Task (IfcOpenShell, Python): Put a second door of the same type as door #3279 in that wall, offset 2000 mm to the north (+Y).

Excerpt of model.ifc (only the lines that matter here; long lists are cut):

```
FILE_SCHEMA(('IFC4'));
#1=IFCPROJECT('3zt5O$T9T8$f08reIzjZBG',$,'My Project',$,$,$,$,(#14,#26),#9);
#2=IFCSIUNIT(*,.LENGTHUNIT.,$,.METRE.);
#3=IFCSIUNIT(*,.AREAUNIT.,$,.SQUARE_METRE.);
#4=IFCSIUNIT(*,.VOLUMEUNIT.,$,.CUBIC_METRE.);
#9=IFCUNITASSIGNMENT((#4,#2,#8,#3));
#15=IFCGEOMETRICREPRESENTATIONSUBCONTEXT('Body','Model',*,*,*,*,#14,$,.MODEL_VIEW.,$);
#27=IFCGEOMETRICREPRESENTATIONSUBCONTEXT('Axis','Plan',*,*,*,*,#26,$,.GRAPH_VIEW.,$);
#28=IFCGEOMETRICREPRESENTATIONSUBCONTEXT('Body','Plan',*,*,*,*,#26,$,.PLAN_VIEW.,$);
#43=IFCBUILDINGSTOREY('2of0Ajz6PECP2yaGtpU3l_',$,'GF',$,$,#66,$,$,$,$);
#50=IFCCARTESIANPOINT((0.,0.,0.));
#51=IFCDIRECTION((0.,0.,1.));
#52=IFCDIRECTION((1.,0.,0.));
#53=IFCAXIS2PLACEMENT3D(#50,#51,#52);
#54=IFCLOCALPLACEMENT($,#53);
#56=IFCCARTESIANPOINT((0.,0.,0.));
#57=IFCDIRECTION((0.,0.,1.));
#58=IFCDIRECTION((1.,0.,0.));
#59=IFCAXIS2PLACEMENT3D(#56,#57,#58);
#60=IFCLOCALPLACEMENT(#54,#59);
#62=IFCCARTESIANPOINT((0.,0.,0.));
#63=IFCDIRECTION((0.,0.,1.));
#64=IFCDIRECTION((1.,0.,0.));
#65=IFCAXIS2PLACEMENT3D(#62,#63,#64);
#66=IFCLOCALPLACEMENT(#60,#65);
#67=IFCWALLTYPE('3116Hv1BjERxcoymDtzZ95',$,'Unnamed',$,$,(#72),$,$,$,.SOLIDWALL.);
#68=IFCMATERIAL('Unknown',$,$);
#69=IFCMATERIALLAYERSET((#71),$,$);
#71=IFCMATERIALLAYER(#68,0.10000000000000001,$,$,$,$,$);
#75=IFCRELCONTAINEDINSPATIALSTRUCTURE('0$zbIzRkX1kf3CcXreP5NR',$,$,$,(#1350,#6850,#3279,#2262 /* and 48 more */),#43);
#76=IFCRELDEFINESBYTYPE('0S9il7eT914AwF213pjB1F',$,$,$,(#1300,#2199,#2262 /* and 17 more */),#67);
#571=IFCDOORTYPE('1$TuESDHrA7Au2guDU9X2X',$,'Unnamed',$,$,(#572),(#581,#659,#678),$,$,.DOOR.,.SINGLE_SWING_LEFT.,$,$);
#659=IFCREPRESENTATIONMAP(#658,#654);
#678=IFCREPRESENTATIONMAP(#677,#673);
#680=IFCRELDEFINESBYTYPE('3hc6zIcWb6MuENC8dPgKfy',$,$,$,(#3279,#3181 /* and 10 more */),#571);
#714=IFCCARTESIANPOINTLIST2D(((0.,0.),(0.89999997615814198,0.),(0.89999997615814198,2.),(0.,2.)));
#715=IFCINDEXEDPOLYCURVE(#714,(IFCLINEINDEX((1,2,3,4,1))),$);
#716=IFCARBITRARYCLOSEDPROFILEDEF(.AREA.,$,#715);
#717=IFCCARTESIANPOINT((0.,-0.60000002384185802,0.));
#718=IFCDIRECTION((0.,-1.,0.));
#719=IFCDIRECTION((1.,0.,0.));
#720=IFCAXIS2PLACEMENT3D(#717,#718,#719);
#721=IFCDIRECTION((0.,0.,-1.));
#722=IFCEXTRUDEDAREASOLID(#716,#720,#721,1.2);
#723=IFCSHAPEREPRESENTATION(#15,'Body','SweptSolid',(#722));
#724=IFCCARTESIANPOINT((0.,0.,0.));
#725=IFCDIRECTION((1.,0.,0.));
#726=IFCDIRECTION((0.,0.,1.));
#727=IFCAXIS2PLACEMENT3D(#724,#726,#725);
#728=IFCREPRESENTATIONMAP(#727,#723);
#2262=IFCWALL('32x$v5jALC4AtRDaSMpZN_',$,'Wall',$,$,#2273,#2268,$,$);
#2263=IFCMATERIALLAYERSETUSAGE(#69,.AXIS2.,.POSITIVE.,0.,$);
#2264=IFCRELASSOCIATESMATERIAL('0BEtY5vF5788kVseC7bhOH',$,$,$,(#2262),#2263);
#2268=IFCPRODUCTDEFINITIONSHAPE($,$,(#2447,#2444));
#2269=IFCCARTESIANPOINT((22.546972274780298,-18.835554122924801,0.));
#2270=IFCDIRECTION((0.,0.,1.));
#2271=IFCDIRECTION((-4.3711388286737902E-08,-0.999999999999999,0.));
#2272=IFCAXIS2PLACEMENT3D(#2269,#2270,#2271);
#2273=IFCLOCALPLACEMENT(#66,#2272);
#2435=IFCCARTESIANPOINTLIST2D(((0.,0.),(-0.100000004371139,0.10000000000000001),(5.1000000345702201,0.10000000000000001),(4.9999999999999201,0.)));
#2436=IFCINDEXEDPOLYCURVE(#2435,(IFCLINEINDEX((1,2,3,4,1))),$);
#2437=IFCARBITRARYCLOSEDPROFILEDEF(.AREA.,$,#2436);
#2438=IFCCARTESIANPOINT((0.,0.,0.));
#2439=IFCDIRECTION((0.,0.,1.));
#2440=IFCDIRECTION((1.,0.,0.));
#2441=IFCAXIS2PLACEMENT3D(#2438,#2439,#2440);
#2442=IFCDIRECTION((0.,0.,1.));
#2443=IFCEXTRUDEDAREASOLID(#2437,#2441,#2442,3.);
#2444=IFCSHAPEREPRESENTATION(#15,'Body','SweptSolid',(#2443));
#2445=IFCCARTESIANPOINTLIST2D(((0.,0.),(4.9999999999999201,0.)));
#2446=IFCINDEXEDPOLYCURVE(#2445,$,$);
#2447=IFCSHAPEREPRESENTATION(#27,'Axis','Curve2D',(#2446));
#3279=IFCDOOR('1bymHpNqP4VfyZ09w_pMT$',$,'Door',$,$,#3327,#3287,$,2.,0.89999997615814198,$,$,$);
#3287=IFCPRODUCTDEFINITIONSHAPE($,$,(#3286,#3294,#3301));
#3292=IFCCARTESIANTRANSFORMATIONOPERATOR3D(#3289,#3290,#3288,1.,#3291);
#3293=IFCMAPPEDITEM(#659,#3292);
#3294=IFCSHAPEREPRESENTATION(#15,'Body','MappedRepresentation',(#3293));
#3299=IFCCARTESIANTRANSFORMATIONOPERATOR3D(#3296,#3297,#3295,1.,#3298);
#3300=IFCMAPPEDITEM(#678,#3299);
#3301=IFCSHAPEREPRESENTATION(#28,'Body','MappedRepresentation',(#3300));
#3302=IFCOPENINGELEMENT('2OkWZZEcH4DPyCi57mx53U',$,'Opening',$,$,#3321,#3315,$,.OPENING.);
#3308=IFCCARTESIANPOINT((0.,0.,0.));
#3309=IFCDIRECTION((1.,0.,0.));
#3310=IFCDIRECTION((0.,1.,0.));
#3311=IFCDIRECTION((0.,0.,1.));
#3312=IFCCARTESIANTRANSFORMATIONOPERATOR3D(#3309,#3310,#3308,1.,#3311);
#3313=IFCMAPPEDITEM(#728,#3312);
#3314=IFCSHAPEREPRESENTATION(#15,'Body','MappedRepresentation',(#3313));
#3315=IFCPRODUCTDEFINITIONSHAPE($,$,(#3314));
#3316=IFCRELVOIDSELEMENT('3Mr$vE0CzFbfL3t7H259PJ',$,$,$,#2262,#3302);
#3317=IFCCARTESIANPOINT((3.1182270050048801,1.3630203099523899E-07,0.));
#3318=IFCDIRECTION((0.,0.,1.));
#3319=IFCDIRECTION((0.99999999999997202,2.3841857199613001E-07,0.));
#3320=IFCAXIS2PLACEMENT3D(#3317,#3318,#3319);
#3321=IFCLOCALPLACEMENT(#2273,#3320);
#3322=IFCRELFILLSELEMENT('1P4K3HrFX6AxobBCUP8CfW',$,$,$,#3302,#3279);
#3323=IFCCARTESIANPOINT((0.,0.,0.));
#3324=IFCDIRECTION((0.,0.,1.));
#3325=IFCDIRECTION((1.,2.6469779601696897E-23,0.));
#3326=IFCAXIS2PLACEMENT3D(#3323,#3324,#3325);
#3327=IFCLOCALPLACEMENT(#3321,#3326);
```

```python
import ifcopenshell
import ifcopenshell.api.feature
import ifcopenshell.api.geometry
import ifcopenshell.api.root
import ifcopenshell.geom
import ifcopenshell.util.element
import ifcopenshell.util.placement
import ifcopenshell.util.shape

model = ifcopenshell.open("model.ifc")
settings = ifcopenshell.geom.settings()


def volume(element):
    """Net volume in cubic metres, openings subtracted."""
    shape = ifcopenshell.geom.create_shape(settings, element)
    return ifcopenshell.util.shape.get_volume(shape.geometry)


door = model.by_id(3279)
opening = door.FillsVoids[0].RelatingOpeningElement
wall = opening.VoidsElements[0].RelatingBuildingElement
before = volume(wall)
shift = ifcopenshell.util.placement.get_local_placement(wall.ObjectPlacement)[:3, 0] * -2.0

# copy_class copies the void relationship, type, container and properties, but no geometry.
new_opening = ifcopenshell.api.root.copy_class(model, product=opening)
new_opening.Representation = ifcopenshell.util.element.copy_deep(
    model, opening.Representation, exclude=["IfcGeometricRepresentationContext", "IfcRepresentationMap"]
)
new_door = ifcopenshell.api.root.copy_class(model, product=door)
new_door.Representation = ifcopenshell.util.element.copy_deep(
    model, door.Representation, exclude=["IfcGeometricRepresentationContext", "IfcRepresentationMap"]
)
ifcopenshell.api.feature.add_filling(model, opening=new_opening, element=new_door)

for old, new in ((opening, new_opening), (door, new_door)):
    matrix = ifcopenshell.util.placement.get_local_placement(old.ObjectPlacement)
    matrix[:3, 3] += shift
    ifcopenshell.api.geometry.edit_object_placement(model, product=new, matrix=matrix, is_si=False)

after = volume(wall)

print(f"wall volume {before:.3f} -> {after:.3f} m3")

model.write("model_edited.ifc")
```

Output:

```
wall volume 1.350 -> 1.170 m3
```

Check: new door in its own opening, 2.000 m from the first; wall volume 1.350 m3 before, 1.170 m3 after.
